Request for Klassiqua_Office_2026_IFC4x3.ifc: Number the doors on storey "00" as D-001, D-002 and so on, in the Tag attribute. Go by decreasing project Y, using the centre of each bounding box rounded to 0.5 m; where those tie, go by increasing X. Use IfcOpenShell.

First a look at what the model holds.

```python
import ifcopenshell
import ifcopenshell.util.element
import ifcopenshell.util.placement

model = ifcopenshell.open("Klassiqua_Office_2026_IFC4x3.ifc")
print(model.schema)
storey = next(s for s in model.by_type("IfcBuildingStorey") if s.Name == "00")
doors = [e for e in ifcopenshell.util.element.get_decomposition(storey) if e.is_a("IfcDoor")]
for e in sorted(doors, key=lambda e: e.id()):
    origin = ifcopenshell.util.placement.get_local_placement(e.ObjectPlacement)[:3, 3]
    print(e.id(), e.Tag, e.Name, origin.round(2) + 0.0, sep=" | ")
```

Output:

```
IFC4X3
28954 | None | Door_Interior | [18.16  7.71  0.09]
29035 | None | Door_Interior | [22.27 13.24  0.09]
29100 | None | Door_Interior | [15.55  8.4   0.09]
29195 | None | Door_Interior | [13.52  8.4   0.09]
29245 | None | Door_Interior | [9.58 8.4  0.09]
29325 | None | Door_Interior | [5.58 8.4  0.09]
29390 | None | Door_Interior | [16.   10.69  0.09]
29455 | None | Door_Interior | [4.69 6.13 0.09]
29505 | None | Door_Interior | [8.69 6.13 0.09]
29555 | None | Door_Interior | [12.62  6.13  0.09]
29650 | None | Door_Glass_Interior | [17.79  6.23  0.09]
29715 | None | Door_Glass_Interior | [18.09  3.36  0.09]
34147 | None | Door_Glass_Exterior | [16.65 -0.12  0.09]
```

```python
import ifcopenshell
import ifcopenshell.geom
import ifcopenshell.util.element
import ifcopenshell.util.shape

model = ifcopenshell.open("Klassiqua_Office_2026_IFC4x3.ifc")
settings = ifcopenshell.geom.settings()
settings.set("use-world-coords", True)


def centre(element):
    shape = ifcopenshell.geom.create_shape(settings, element)
    return ifcopenshell.util.shape.get_bbox_centroid(shape.geometry)


storey = next(s for s in model.by_type("IfcBuildingStorey") if s.Name == "00")
doors = [e for e in ifcopenshell.util.element.get_decomposition(storey) if e.is_a("IfcDoor")]

# Insertion points can sit at a corner or the storey origin, so sort by the geometry (in metres).
centres = {e: centre(e) for e in doors}
doors.sort(key=lambda e: (-round(centres[e][1] / 0.5), centres[e][0]))

for i, e in enumerate(doors, start=1):
    number = f"D-0{i:02d}"
    e.Tag = number
    print(e.id(), number)

model.write("Klassiqua_Office_2026_IFC4x3_v2.ifc")
```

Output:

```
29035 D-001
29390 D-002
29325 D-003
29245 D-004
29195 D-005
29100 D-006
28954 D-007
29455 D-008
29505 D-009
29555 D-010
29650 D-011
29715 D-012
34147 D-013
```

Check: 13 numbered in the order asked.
